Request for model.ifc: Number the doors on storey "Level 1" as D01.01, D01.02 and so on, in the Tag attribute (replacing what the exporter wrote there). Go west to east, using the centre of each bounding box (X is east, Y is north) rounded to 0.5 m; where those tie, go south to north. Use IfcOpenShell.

First a look at what the model holds.

```python
import ifcopenshell
import ifcopenshell.util.element
import ifcopenshell.util.placement

model = ifcopenshell.open("model.ifc")
print(model.schema)
storey = next(s for s in model.by_type("IfcBuildingStorey") if s.Name == "Level 1")
doors = [e for e in ifcopenshell.util.element.get_decomposition(storey) if e.is_a("IfcDoor")]
for e in sorted(doors, key=lambda e: e.id()):
    origin = ifcopenshell.util.placement.get_local_placement(e.ObjectPlacement)[:3, 3]
    print(e.id(), e.Tag, e.Name, origin.round(2) + 0.0, sep=" | ")
```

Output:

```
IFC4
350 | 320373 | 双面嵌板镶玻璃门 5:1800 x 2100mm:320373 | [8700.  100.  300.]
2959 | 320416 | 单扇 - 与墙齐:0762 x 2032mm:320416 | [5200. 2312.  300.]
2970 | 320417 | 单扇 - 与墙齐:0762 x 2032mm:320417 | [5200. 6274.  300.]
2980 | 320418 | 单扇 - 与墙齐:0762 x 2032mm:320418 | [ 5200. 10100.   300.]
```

```python
import ifcopenshell
import ifcopenshell.geom
import ifcopenshell.util.element
import ifcopenshell.util.shape

model = ifcopenshell.open("model.ifc")
settings = ifcopenshell.geom.settings()
settings.set("use-world-coords", True)


def centre(element):
    shape = ifcopenshell.geom.create_shape(settings, element)
    return ifcopenshell.util.shape.get_bbox_centroid(shape.geometry)


storey = next(s for s in model.by_type("IfcBuildingStorey") if s.Name == "Level 1")
doors = [e for e in ifcopenshell.util.element.get_decomposition(storey) if e.is_a("IfcDoor")]

# Insertion points can sit at a corner or the storey origin, so sort by the geometry (in metres).
centres = {e: centre(e) for e in doors}
doors.sort(key=lambda e: (round(centres[e][0] / 0.5), centres[e][1]))

for i, e in enumerate(doors, start=1):
    number = f"D01.{i:02d}"
    e.Tag = number
    print(e.id(), number)

model.write("model_edited.ifc")
```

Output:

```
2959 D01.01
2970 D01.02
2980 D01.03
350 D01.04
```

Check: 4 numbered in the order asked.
